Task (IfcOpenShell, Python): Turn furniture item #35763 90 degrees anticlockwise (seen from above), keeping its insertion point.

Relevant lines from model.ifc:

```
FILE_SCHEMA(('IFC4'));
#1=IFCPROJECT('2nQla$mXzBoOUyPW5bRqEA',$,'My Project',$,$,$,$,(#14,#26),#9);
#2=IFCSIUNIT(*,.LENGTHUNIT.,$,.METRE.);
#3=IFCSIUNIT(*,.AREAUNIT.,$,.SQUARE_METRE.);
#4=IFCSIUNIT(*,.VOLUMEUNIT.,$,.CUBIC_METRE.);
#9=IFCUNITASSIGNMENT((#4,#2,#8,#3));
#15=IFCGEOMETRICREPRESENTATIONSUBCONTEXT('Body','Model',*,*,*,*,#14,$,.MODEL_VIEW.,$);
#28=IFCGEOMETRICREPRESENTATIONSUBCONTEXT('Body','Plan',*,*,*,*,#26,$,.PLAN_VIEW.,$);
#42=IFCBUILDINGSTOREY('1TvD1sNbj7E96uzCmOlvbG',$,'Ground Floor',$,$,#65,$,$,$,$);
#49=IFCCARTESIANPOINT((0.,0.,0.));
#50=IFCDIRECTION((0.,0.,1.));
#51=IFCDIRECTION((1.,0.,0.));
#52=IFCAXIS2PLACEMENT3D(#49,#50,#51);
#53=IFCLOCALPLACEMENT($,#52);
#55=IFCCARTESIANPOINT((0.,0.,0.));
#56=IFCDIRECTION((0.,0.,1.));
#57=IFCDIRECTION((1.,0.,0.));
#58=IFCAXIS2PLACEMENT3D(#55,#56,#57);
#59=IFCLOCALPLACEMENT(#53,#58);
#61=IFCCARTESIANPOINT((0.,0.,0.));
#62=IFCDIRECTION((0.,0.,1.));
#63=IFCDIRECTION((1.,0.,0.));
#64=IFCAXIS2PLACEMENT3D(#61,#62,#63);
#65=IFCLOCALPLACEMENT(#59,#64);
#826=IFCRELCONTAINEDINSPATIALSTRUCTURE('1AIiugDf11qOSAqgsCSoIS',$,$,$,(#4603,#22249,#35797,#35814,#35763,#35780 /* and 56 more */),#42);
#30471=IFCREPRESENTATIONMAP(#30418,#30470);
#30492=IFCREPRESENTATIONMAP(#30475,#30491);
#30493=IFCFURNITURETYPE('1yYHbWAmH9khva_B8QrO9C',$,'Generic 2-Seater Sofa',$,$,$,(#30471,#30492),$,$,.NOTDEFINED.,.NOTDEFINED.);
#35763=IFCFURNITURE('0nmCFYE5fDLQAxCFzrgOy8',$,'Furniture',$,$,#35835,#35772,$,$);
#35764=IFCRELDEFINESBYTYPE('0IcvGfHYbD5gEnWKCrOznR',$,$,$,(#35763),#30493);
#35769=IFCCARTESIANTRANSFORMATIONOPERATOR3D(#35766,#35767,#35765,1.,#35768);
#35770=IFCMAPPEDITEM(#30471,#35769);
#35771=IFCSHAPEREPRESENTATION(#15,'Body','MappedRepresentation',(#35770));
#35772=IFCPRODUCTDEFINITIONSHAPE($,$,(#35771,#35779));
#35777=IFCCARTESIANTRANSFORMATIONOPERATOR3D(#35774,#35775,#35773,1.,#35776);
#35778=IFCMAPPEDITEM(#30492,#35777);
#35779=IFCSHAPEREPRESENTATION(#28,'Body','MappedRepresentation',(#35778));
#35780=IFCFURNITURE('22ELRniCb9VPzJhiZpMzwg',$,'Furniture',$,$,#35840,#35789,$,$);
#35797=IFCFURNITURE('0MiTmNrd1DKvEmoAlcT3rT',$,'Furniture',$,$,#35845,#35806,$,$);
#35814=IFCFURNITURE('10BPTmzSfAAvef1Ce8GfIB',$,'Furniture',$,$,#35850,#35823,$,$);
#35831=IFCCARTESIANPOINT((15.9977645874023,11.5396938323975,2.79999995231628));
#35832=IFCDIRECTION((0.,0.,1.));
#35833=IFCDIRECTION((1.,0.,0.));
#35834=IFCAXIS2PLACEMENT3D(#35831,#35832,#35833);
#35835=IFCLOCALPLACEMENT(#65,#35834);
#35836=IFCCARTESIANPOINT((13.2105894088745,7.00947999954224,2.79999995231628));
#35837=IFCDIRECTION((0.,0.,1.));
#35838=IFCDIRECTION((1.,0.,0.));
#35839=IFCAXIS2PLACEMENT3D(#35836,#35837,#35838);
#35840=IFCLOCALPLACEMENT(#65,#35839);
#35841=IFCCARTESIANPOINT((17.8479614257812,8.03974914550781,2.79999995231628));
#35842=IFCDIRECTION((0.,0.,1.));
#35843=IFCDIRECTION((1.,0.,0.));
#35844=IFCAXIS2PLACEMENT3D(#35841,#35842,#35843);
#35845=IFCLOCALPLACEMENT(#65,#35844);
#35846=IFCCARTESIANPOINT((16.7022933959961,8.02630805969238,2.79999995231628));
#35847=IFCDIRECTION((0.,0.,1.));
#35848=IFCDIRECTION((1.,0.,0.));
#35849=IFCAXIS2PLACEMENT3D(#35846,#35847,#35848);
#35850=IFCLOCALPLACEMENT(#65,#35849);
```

```python
import ifcopenshell
import ifcopenshell.api.geometry
import ifcopenshell.util.placement

model = ifcopenshell.open("model.ifc")

item = model.by_guid("0nmCFYE5fDLQAxCFzrgOy8")
matrix = ifcopenshell.util.placement.get_local_placement(item.ObjectPlacement)
matrix = matrix @ ifcopenshell.util.placement.rotation(90, "Z")
ifcopenshell.api.geometry.edit_object_placement(model, product=item, matrix=matrix, is_si=False)

print(ifcopenshell.util.placement.get_local_placement(item.ObjectPlacement).round(3) + 0.0)

model.write("model_updated.ifc")
```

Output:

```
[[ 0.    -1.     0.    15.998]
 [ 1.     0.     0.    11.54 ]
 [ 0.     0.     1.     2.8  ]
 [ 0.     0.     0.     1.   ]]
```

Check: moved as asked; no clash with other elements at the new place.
